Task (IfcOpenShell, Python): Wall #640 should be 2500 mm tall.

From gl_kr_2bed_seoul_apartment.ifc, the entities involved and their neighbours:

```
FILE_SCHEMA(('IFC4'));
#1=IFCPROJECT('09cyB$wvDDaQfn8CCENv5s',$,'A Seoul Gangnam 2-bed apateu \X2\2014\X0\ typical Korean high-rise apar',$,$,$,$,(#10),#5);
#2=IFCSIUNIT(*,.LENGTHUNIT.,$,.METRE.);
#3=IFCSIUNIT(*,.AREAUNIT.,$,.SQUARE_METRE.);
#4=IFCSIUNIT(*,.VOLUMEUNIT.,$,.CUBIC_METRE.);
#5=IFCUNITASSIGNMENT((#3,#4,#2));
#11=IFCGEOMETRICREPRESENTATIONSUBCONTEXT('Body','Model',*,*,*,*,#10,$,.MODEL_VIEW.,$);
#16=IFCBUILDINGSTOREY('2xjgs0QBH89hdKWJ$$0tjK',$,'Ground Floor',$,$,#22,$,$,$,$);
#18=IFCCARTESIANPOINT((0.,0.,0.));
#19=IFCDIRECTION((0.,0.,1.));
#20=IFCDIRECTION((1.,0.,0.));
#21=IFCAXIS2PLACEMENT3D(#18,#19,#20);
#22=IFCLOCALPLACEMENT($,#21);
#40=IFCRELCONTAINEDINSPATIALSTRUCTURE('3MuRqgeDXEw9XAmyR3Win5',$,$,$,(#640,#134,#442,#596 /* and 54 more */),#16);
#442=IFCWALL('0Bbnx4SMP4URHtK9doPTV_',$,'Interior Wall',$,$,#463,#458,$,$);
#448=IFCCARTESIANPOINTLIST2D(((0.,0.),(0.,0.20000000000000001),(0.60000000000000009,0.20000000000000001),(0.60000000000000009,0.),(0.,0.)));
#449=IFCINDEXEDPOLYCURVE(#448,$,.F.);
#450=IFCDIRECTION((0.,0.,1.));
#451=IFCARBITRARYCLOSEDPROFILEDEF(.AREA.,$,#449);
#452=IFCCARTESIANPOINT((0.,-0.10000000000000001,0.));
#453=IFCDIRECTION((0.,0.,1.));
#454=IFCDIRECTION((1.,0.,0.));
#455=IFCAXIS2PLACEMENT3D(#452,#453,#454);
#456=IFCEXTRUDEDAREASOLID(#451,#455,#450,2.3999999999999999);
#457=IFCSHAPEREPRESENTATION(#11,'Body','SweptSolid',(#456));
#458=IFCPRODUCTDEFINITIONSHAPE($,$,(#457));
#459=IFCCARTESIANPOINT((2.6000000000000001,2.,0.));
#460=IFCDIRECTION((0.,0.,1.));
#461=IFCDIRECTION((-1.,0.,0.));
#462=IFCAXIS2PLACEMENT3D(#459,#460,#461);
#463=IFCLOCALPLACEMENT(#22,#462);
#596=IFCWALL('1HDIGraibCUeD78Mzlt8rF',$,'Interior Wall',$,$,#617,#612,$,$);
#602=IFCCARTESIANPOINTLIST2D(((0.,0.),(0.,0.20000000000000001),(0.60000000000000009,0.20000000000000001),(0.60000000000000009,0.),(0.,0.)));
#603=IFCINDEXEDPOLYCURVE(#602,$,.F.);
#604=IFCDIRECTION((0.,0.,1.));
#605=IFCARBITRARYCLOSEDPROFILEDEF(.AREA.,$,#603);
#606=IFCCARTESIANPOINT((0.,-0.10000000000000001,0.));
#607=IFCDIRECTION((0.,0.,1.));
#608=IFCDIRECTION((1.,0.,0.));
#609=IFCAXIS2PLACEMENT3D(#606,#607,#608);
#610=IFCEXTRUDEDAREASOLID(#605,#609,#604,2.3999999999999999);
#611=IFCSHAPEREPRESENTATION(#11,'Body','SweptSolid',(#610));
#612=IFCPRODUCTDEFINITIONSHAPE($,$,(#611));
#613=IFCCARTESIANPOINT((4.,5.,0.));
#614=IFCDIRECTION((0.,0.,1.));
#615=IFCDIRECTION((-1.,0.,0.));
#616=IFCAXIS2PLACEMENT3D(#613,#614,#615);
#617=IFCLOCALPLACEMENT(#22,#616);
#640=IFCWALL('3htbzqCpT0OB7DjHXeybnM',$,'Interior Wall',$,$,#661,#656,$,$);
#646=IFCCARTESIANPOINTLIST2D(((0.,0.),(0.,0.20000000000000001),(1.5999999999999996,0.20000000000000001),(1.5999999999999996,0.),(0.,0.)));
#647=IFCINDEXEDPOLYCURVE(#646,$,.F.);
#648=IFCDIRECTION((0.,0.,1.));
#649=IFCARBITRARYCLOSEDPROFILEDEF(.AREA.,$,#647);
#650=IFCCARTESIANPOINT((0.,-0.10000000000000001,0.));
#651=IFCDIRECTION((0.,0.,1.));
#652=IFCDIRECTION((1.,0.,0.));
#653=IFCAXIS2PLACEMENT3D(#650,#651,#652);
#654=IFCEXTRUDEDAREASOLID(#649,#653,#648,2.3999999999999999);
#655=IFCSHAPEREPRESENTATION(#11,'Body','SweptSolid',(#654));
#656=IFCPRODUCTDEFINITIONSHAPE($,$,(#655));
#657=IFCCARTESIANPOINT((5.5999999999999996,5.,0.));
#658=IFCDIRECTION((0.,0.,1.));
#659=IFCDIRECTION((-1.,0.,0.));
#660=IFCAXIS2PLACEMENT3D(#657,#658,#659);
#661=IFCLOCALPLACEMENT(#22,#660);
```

```python
import ifcopenshell
import ifcopenshell.geom
import ifcopenshell.util.representation
import ifcopenshell.util.shape

model = ifcopenshell.open("gl_kr_2bed_seoul_apartment.ifc")
settings = ifcopenshell.geom.settings()


def volume(element):
    """Net volume in cubic metres, openings subtracted."""
    shape = ifcopenshell.geom.create_shape(settings, element)
    return ifcopenshell.util.shape.get_volume(shape.geometry)


wall = model.by_id(640)
before = volume(wall)

body = ifcopenshell.util.representation.get_representation(wall, "Model", "Body")
solid = body.Items[0]
old_height = solid.Depth
solid.Depth = 2.5
after = volume(wall)

print(f"height {old_height:g} -> {solid.Depth:g}, volume {before:.3f} -> {after:.3f} m3")

model.write("gl_kr_2bed_seoul_apartment_rev.ifc")
```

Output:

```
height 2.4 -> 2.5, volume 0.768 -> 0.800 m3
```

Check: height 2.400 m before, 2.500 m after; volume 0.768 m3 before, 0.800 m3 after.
